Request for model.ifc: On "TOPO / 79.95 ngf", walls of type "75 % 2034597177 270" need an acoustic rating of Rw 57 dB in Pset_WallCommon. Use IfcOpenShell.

First a look at what the model holds.

```python
import ifcopenshell
import ifcopenshell.util.element

model = ifcopenshell.open("model.ifc")
print(model.schema)
storey = next(s for s in model.by_type("IfcBuildingStorey") if s.Name == "TOPO / 79.95 ngf")
walls = [e for e in ifcopenshell.util.element.get_decomposition(storey) if e.is_a("IfcWall")]
seen = {}
for e in walls:
    element_type = ifcopenshell.util.element.get_type(e)
    key = (element_type.Name if element_type != e and element_type else None, ifcopenshell.util.element.get_pset(e, "Pset_WallCommon", "AcousticRating"))
    seen[key] = seen.get(key, 0) + 1
for (name, value), count in sorted(seen.items(), key=str):
    print(count, "x", name, "|", value)
```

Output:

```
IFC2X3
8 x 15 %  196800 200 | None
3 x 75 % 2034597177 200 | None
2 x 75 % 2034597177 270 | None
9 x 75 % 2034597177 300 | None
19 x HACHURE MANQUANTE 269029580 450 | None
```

```python
import ifcopenshell
import ifcopenshell.api.pset
import ifcopenshell.util.element

model = ifcopenshell.open("model.ifc")

storey = next(s for s in model.by_type("IfcBuildingStorey") if s.Name == "TOPO / 79.95 ngf")
walls = [e for e in ifcopenshell.util.element.get_decomposition(storey) if e.is_a("IfcWall")]

count = 0
for e in walls:
    element_type = ifcopenshell.util.element.get_type(e)
    if element_type in (None, e) or element_type.Name != "75 % 2034597177 270":
        continue
    # add_pset returns the element's existing set when there is one.
    pset = ifcopenshell.api.pset.add_pset(model, product=e, name="Pset_WallCommon")
    ifcopenshell.api.pset.edit_pset(model, pset=pset, properties={"AcousticRating": "Rw 57 dB"})
    count += 1

print(count, "walls updated")

model.write("model_v2.ifc")
```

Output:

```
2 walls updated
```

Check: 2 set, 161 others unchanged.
